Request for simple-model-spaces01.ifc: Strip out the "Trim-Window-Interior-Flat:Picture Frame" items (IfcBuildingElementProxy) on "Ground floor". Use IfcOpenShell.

First a look at what the model holds.

```python
import ifcopenshell
import ifcopenshell.util.element

model = ifcopenshell.open("simple-model-spaces01.ifc")
print(model.schema)
storey = next(s for s in model.by_type("IfcBuildingStorey") if s.Name == "Ground floor")
proxies = [e for e in ifcopenshell.util.element.get_decomposition(storey) if e.is_a("IfcBuildingElementProxy")]
seen = {}
for e in proxies:
    element_type = ifcopenshell.util.element.get_type(e)
    name = element_type.Name if element_type not in (None, e) else None
    seen[name] = seen.get(name, 0) + 1
for name, count in sorted(seen.items(), key=str):
    print(count, "x", name)
```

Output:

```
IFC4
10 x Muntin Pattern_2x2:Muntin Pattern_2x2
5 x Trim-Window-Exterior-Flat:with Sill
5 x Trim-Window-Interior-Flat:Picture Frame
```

```python
import ifcopenshell
import ifcopenshell.api.root
import ifcopenshell.util.element

model = ifcopenshell.open("simple-model-spaces01.ifc")

storey = next(s for s in model.by_type("IfcBuildingStorey") if s.Name == "Ground floor")
proxies = [e for e in ifcopenshell.util.element.get_decomposition(storey) if e.is_a("IfcBuildingElementProxy")]
targets = [e for e in proxies if (t := ifcopenshell.util.element.get_type(e)) not in (None, e) and t.Name == "Trim-Window-Interior-Flat:Picture Frame"]

for e in targets:
    ifcopenshell.api.root.remove_product(model, product=e)
print(len(targets), "removed")

model.write("simple-model-spaces01_rev.ifc")
```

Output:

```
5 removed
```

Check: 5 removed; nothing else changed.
